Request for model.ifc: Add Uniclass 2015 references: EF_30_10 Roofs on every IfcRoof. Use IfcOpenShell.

First a look at what the model holds.

```python
import ifcopenshell

model = ifcopenshell.open("model.ifc")
print(model.schema)
print("classifications:", [c.Name for c in model.by_type("IfcClassification")])
for ifc_class in ("IfcDoor", "IfcRoof", "IfcStair", "IfcWall", "IfcWindow"):
    print(ifc_class, len(model.by_type(ifc_class)))
```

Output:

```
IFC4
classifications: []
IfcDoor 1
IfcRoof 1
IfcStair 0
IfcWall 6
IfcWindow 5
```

```python
import ifcopenshell
import ifcopenshell.api.classification

model = ifcopenshell.open("model.ifc")

system = ifcopenshell.api.classification.add_classification(model, classification="Uniclass 2015")

codes = {
    "IfcRoof": ("EF_30_10", "Roofs"),
}
for ifc_class, (code, name) in codes.items():
    products = model.by_type(ifc_class)
    ifcopenshell.api.classification.add_reference(
        model, products=products, classification=system, identification=code, name=name
    )
    print(code, len(products))

model.write("model_updated.ifc")
```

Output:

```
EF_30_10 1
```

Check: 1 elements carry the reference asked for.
